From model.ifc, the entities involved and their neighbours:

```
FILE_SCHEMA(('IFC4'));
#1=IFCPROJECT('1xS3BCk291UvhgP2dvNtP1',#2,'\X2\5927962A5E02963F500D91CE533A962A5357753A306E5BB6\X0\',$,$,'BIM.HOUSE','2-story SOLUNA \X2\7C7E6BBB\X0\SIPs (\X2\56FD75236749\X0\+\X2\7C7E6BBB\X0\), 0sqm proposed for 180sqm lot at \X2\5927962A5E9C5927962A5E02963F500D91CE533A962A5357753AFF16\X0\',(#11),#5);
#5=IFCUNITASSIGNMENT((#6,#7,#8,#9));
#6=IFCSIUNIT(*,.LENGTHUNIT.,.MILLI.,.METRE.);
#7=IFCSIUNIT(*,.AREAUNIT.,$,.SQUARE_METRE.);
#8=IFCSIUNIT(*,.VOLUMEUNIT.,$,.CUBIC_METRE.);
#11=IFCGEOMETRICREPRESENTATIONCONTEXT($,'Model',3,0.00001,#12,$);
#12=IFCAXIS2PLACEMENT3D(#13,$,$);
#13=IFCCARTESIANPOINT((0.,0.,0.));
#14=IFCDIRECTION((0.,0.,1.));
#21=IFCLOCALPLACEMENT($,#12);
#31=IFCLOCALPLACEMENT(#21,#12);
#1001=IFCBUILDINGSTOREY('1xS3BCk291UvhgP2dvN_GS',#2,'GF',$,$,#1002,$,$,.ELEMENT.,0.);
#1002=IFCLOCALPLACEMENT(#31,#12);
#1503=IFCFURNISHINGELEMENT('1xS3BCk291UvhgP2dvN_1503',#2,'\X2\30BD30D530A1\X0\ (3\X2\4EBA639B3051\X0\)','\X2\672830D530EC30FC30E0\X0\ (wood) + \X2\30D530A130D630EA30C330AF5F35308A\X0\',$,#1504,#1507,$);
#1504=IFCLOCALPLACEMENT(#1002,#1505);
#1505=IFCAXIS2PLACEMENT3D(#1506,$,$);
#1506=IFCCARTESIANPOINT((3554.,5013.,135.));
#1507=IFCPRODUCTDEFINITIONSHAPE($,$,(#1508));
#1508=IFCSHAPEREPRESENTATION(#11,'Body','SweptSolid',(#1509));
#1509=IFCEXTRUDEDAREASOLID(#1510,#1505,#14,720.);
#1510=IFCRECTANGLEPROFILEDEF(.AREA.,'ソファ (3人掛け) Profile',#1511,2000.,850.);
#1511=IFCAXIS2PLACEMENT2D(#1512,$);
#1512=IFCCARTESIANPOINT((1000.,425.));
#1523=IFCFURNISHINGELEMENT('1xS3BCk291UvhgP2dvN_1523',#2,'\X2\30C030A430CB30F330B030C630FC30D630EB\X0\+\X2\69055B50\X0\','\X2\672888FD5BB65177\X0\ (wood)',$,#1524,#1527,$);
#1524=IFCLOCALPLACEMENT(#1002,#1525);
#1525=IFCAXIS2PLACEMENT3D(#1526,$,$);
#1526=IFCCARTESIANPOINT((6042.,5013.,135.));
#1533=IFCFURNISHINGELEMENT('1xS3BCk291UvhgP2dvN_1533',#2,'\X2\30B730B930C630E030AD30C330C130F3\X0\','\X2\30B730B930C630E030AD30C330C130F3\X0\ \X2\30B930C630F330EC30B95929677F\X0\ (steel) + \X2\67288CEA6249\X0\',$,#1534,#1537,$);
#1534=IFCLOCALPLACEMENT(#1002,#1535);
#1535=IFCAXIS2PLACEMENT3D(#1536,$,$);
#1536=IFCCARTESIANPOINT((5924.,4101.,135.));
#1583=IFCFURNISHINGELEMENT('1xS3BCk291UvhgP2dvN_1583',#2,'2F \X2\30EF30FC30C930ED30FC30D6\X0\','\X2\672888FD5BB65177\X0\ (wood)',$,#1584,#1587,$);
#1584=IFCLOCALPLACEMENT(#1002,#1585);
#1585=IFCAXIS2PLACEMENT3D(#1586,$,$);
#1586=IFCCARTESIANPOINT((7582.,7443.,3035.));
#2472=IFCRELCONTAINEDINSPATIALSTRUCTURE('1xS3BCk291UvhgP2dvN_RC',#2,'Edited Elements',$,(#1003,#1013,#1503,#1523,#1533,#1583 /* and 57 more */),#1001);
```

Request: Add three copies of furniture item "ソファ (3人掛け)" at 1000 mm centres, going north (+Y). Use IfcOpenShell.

```python
import numpy as np
import ifcopenshell
import ifcopenshell.api.geometry
import ifcopenshell.api.root
import ifcopenshell.util.element
import ifcopenshell.util.placement
import ifcopenshell.util.unit

model = ifcopenshell.open("model.ifc")
unit_scale = ifcopenshell.util.unit.calculate_unit_scale(model)


def reuse_history(source, copy):
    """copy_class also copies each property set's owner history, people and application; keep the originals."""
    for rel in copy.IsDefinedBy:
        if rel.is_a("IfcRelDefinesByProperties") and (history := rel.RelatingPropertyDefinition.OwnerHistory):
            rel.RelatingPropertyDefinition.OwnerHistory = source.OwnerHistory
            ifcopenshell.util.element.remove_deep2(model, history)


source = model.by_id(1503)
base = ifcopenshell.util.placement.get_local_placement(source.ObjectPlacement)
step = np.array([0.0, 1.0, 0.0]) * 1 / unit_scale

for i in range(1, 4):
    copy = ifcopenshell.api.root.copy_class(model, product=source)
    copy.Representation = ifcopenshell.util.element.copy_deep(
        model, source.Representation, exclude=["IfcGeometricRepresentationContext", "IfcRepresentationMap"]
    )
    reuse_history(source, copy)
    matrix = base.copy()
    matrix[:3, 3] += i * step
    print("added at", matrix[:3, 3].round(3) + 0.0)
    ifcopenshell.api.geometry.edit_object_placement(model, product=copy, matrix=matrix, is_si=False)

model.write("model-out.ifc")
```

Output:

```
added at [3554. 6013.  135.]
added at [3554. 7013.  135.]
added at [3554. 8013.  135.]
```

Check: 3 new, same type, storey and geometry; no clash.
